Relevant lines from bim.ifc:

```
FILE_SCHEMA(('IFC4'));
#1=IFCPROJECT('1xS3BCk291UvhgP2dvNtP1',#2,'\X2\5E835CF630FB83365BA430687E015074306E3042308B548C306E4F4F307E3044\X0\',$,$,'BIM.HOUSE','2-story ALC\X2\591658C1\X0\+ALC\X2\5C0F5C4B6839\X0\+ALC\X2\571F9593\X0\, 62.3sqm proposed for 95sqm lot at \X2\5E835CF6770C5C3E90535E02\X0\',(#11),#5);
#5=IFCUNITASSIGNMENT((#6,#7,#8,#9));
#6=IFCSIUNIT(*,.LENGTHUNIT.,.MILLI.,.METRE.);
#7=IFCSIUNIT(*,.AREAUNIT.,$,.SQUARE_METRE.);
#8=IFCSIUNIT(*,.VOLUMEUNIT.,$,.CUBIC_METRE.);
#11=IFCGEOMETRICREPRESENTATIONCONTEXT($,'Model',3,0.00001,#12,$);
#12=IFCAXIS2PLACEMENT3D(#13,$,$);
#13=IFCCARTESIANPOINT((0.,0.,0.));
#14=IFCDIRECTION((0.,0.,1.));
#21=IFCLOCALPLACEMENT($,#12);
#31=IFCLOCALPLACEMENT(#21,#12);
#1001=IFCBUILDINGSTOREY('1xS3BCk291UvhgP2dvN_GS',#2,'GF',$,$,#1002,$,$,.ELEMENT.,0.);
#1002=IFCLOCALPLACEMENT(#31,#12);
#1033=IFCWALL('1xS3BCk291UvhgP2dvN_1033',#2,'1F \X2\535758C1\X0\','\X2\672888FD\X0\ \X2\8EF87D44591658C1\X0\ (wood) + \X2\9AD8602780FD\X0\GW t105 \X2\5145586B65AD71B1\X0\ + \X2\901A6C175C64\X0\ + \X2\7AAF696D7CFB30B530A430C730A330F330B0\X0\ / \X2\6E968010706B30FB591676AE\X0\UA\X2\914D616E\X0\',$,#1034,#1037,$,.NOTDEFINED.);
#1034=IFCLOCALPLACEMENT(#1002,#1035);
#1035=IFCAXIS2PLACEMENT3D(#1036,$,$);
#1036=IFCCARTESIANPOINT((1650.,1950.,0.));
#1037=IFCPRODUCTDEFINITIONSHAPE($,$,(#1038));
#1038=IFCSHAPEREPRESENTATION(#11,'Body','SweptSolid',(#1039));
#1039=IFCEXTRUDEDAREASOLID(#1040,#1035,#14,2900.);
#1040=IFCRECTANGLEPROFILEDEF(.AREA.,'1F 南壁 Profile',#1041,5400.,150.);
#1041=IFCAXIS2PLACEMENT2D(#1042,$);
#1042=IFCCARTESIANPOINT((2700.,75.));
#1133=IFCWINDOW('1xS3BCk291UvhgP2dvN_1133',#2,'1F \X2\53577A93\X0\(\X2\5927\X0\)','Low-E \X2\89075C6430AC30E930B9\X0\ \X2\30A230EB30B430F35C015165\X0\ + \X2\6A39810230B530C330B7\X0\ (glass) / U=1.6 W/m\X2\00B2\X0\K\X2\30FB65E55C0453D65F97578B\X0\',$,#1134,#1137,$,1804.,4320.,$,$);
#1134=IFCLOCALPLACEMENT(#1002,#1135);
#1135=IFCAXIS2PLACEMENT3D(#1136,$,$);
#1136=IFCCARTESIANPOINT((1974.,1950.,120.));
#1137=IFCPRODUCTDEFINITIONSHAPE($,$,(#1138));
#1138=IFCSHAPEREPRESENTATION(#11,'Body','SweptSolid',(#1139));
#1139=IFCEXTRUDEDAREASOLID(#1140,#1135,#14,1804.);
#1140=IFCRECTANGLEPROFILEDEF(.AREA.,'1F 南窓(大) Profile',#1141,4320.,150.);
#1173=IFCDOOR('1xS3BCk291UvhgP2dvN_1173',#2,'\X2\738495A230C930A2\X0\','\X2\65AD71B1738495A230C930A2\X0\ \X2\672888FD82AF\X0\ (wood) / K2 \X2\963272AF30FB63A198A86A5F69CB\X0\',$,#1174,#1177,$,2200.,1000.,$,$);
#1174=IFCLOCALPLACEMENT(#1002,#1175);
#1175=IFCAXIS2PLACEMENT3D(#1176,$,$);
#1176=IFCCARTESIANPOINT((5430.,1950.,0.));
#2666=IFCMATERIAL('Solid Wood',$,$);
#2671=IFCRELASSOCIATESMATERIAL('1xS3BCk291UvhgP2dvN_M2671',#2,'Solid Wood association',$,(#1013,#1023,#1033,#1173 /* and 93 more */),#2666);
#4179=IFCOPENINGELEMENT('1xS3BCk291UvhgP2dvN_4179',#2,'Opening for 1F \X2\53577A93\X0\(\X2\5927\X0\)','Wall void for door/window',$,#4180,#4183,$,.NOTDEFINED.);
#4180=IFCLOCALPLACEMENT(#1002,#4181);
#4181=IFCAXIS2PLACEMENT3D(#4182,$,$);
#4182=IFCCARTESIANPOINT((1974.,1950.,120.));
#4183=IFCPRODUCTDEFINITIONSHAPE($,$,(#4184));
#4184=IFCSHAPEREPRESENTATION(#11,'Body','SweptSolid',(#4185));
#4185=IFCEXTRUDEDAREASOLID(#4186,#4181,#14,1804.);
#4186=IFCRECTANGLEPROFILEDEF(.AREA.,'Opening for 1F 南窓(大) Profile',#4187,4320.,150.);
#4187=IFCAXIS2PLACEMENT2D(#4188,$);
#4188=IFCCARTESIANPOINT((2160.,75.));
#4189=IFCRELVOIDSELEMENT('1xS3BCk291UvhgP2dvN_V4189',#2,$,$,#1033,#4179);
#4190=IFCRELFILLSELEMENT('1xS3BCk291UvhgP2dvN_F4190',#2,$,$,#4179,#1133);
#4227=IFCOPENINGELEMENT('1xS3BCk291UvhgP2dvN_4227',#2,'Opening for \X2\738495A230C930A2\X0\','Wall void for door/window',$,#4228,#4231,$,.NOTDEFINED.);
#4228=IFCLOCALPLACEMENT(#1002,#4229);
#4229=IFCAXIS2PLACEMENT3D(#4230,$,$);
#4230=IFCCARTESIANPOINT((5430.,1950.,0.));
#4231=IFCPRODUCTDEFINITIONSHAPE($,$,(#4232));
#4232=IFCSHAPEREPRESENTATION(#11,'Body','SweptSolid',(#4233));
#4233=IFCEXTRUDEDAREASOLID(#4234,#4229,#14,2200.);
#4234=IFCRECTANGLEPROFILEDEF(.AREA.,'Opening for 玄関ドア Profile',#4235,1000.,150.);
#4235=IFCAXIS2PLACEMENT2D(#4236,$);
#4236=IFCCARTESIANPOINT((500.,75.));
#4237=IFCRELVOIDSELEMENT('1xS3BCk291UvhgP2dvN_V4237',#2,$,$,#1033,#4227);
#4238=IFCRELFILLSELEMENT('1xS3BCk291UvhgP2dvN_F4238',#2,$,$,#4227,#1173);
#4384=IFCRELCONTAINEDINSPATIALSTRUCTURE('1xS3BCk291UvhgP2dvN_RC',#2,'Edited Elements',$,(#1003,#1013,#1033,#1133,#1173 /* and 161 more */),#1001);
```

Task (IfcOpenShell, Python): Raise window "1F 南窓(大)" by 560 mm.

```python
import numpy as np
import ifcopenshell
import ifcopenshell.api.geometry
import ifcopenshell.util.placement
import ifcopenshell.util.unit

model = ifcopenshell.open("bim.ifc")
unit_scale = ifcopenshell.util.unit.calculate_unit_scale(model)

window = model.by_guid("1xS3BCk291UvhgP2dvN_1133")
opening = window.FillsVoids[0].RelatingOpeningElement
dz = 0.56 / unit_scale

shift = np.array([0.0, 0.0, dz])
# The window is not placed relative to its opening, so move both.
for product in (opening, window):
    matrix = ifcopenshell.util.placement.get_local_placement(product.ObjectPlacement)
    matrix[:3, 3] += shift
    ifcopenshell.api.geometry.edit_object_placement(model, product=product, matrix=matrix, is_si=False)

print(f"moved by {dz * unit_scale:+.3f} m")

model.write("bim_edited.ifc")
```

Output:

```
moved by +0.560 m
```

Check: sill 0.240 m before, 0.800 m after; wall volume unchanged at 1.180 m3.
